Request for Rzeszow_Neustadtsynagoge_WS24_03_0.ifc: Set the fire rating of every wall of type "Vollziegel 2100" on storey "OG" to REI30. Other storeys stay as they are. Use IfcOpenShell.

First a look at what the model holds.

```python
import ifcopenshell
import ifcopenshell.util.element

model = ifcopenshell.open("Rzeszow_Neustadtsynagoge_WS24_03_0.ifc")
print(model.schema)
storey = next(s for s in model.by_type("IfcBuildingStorey") if s.Name == "OG")
walls = [e for e in ifcopenshell.util.element.get_decomposition(storey) if e.is_a("IfcWall")]
seen = {}
for e in walls:
    element_type = ifcopenshell.util.element.get_type(e)
    key = (element_type.Name if element_type != e and element_type else None, ifcopenshell.util.element.get_pset(e, "Pset_WallCommon", "FireRating"))
    seen[key] = seen.get(key, 0) + 1
for (name, value), count in sorted(seen.items(), key=str):
    print(count, "x", name, "|", value)
```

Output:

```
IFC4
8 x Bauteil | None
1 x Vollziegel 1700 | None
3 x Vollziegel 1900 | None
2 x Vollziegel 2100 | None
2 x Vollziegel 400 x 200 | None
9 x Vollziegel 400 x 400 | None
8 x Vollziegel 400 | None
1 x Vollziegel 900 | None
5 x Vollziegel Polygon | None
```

```python
import ifcopenshell
import ifcopenshell.api.pset
import ifcopenshell.util.element

model = ifcopenshell.open("Rzeszow_Neustadtsynagoge_WS24_03_0.ifc")

storey = next(s for s in model.by_type("IfcBuildingStorey") if s.Name == "OG")
walls = [e for e in ifcopenshell.util.element.get_decomposition(storey) if e.is_a("IfcWall")]

count = 0
for e in walls:
    element_type = ifcopenshell.util.element.get_type(e)
    if element_type in (None, e) or element_type.Name != "Vollziegel 2100":
        continue
    # add_pset returns the element's existing set when there is one.
    pset = ifcopenshell.api.pset.add_pset(model, product=e, name="Pset_WallCommon")
    ifcopenshell.api.pset.edit_pset(model, pset=pset, properties={"FireRating": "REI30"})
    count += 1

print(count, "walls updated")

model.write("Rzeszow_Neustadtsynagoge_WS24_03_0_v2.ifc")
```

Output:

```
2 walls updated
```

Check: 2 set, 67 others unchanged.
